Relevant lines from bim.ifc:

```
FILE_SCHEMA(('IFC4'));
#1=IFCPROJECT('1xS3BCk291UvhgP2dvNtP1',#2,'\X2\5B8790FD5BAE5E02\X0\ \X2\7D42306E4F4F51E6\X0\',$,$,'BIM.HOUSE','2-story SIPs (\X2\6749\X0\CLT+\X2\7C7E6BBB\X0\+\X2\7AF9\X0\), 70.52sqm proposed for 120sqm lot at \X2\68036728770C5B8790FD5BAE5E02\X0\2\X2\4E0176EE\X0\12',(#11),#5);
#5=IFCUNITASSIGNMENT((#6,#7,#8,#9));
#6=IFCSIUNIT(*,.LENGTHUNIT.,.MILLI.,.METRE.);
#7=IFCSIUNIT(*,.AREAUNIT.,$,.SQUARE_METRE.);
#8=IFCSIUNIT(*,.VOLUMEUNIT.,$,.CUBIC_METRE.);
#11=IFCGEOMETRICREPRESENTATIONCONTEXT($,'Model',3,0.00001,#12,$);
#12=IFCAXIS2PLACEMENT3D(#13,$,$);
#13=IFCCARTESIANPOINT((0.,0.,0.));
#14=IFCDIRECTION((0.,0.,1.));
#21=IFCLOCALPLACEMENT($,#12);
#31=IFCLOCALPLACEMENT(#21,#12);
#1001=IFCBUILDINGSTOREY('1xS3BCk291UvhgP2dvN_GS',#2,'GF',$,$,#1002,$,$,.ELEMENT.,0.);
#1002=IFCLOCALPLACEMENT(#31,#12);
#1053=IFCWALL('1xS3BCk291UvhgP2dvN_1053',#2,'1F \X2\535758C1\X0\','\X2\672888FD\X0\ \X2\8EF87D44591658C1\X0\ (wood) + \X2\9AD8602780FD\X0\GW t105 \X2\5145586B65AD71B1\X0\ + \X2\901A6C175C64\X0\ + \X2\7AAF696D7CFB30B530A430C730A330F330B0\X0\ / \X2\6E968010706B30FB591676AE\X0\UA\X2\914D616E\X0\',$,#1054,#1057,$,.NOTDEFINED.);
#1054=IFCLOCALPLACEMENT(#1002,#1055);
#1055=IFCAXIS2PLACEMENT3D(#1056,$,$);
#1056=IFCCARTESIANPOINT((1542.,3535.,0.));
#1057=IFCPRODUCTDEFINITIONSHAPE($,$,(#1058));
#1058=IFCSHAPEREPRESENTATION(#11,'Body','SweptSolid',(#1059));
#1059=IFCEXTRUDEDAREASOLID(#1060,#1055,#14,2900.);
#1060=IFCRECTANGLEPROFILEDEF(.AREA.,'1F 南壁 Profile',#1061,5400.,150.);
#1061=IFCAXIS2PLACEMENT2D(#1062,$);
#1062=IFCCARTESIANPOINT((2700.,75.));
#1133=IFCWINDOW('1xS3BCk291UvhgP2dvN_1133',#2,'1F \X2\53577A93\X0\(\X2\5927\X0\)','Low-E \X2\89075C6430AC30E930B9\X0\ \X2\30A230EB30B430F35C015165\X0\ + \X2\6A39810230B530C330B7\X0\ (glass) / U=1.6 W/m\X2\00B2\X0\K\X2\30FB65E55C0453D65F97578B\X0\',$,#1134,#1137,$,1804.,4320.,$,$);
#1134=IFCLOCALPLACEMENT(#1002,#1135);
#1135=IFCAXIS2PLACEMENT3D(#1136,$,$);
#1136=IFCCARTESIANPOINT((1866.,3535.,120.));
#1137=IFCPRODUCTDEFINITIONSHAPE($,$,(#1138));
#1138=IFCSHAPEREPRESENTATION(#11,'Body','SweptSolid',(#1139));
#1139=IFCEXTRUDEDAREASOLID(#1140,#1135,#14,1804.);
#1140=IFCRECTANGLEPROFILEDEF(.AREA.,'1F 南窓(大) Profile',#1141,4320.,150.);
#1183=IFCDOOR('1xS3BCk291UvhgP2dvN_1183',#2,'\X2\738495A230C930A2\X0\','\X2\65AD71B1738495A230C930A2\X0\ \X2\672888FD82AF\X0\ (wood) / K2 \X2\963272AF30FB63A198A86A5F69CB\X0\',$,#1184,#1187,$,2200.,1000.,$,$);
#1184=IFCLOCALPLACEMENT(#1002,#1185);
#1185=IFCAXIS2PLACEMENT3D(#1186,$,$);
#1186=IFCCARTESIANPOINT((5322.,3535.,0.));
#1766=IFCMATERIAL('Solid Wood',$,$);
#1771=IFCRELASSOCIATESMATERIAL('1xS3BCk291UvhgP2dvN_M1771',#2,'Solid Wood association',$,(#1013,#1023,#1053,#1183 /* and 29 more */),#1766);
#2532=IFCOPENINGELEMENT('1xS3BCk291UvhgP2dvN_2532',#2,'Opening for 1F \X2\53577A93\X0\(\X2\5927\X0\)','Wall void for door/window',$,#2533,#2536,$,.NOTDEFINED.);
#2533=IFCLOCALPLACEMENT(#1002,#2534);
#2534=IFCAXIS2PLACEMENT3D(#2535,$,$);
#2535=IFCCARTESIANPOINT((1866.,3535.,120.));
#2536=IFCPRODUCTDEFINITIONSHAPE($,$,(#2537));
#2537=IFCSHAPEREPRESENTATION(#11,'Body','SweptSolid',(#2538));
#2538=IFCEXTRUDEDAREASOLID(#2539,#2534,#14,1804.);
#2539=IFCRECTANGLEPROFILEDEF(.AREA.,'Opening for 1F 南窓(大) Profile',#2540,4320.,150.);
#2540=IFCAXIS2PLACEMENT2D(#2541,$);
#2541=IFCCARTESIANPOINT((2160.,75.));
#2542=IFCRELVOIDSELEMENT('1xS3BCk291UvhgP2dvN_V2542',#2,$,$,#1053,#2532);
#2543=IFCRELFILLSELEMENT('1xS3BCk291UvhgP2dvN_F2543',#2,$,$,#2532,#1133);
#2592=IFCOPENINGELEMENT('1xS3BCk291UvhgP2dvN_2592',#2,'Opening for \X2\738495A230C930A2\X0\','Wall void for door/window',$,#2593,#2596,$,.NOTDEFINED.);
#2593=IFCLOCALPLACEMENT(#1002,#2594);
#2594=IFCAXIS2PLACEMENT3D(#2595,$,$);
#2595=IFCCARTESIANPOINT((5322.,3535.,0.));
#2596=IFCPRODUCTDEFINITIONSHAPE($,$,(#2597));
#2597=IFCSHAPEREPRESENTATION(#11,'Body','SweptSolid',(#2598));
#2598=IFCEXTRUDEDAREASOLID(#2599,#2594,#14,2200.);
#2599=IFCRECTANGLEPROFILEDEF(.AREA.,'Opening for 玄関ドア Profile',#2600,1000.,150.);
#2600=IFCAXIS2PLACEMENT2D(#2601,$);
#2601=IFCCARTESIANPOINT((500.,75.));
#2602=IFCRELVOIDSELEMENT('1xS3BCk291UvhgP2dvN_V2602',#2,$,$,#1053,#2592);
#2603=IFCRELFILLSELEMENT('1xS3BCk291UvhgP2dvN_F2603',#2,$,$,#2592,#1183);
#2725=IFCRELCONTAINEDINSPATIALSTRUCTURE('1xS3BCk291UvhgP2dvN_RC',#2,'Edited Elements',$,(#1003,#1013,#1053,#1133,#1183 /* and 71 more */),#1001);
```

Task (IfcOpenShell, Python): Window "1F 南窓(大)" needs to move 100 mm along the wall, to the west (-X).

```python
import ifcopenshell
import ifcopenshell.api.geometry
import ifcopenshell.util.placement
import ifcopenshell.util.unit

model = ifcopenshell.open("bim.ifc")
unit_scale = ifcopenshell.util.unit.calculate_unit_scale(model)

window = model.by_guid("1xS3BCk291UvhgP2dvN_1133")
opening = window.FillsVoids[0].RelatingOpeningElement
wall = opening.VoidsElements[0].RelatingBuildingElement

wall_matrix = ifcopenshell.util.placement.get_local_placement(wall.ObjectPlacement)
shift = wall_matrix[:3, 0] * -0.1 / unit_scale
before = ifcopenshell.util.placement.get_local_placement(window.ObjectPlacement)[:3, 3].copy()

# The window is not placed relative to its opening, so move both.
for product in (opening, window):
    matrix = ifcopenshell.util.placement.get_local_placement(product.ObjectPlacement)
    matrix[:3, 3] += shift
    ifcopenshell.api.geometry.edit_object_placement(model, product=product, matrix=matrix, is_si=False)

after = ifcopenshell.util.placement.get_local_placement(window.ObjectPlacement)[:3, 3]
print("window moved by", (after - before).round(3) + 0.0)

model.write("bim_updated.ifc")
```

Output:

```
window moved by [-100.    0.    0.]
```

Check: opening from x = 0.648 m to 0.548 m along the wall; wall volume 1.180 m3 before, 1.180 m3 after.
